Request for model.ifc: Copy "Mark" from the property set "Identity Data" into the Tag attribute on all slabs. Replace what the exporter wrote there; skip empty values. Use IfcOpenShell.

First a look at what the model holds.

```python
import ifcopenshell
import ifcopenshell.util.element

model = ifcopenshell.open("model.ifc")
print(model.schema)
slabs = model.by_type("IfcSlab")
print(len(slabs), "slabs")
for e in slabs[:8]:
    source = ifcopenshell.util.element.get_pset(e, "Identity Data", "Mark")
    target = e.Tag
    print(e.id(), repr(source), repr(target), sep=" | ")
```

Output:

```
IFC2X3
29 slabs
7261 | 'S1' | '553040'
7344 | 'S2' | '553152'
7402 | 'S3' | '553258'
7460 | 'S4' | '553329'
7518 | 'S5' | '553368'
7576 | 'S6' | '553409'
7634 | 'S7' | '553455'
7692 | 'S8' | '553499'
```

```python
import ifcopenshell
import ifcopenshell.util.element

model = ifcopenshell.open("model.ifc")

count = 0
for e in model.by_type("IfcSlab"):
    value = ifcopenshell.util.element.get_pset(e, "Identity Data", "Mark")
    current = e.Tag
    if not value or not value.strip() or current == value:
        continue
    e.Tag = value
    count += 1

print(count, "slabs updated")

model.write("model-out.ifc")
```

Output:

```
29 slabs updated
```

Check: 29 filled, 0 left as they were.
